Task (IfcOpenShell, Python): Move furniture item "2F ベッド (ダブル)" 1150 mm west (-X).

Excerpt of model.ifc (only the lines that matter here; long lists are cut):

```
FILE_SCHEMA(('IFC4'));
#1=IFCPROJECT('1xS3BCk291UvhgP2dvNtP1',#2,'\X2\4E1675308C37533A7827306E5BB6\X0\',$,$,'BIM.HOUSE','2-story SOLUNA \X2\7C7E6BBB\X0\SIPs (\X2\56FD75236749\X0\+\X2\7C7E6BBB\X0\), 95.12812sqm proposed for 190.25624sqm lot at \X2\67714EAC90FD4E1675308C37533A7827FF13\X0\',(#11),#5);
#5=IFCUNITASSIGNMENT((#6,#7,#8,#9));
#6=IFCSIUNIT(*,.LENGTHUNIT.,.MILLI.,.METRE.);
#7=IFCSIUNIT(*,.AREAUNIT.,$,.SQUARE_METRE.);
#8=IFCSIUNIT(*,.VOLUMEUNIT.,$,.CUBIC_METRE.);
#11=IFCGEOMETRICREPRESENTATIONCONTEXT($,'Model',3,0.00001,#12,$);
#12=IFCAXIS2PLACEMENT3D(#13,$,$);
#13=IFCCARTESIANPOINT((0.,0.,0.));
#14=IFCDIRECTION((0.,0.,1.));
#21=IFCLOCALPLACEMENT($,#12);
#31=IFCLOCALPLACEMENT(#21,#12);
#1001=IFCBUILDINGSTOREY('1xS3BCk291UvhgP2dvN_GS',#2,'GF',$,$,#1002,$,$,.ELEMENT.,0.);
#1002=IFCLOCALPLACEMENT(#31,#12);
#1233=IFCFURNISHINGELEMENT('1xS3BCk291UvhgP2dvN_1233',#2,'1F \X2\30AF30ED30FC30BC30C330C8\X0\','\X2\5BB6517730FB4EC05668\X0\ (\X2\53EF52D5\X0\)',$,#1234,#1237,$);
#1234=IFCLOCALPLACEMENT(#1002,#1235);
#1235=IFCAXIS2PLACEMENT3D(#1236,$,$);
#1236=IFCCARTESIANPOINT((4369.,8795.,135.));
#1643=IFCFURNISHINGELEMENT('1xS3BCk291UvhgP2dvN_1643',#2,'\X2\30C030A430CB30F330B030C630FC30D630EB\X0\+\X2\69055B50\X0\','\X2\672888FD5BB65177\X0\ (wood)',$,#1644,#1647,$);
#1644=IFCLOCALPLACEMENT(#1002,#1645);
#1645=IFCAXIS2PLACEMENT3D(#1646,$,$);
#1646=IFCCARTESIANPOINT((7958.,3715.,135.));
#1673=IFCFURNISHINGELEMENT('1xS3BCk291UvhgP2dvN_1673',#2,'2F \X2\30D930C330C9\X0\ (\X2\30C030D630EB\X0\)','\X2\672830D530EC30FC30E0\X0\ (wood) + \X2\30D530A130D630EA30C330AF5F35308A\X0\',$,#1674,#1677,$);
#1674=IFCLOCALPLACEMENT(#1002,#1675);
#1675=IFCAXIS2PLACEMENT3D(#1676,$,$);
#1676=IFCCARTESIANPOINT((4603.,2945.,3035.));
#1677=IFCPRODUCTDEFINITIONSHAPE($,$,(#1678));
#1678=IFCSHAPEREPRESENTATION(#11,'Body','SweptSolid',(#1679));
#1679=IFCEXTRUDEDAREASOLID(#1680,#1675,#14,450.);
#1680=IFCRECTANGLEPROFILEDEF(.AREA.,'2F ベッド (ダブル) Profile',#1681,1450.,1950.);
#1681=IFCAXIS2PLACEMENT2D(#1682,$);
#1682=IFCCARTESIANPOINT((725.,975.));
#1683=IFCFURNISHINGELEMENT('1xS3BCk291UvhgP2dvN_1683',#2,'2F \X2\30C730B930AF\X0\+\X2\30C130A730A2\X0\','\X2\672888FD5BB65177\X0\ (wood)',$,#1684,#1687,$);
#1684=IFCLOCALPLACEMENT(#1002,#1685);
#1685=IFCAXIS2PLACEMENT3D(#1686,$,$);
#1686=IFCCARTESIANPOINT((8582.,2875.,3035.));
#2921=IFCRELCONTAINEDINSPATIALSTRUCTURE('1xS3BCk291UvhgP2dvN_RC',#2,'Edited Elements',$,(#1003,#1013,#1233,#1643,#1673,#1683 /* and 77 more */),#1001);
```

```python
import ifcopenshell
import ifcopenshell.api.geometry
import ifcopenshell.util.placement

model = ifcopenshell.open("model.ifc")

item = model.by_guid("1xS3BCk291UvhgP2dvN_1673")
matrix = ifcopenshell.util.placement.get_local_placement(item.ObjectPlacement)
matrix[0, 3] -= 1150.0
ifcopenshell.api.geometry.edit_object_placement(model, product=item, matrix=matrix, is_si=False)

print(ifcopenshell.util.placement.get_local_placement(item.ObjectPlacement).round(3) + 0.0)

model.write("model_rev.ifc")
```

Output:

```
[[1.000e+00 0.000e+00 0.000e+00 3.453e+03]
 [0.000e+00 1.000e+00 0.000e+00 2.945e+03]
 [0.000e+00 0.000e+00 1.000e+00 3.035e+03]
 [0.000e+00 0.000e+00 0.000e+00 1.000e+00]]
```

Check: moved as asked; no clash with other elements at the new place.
